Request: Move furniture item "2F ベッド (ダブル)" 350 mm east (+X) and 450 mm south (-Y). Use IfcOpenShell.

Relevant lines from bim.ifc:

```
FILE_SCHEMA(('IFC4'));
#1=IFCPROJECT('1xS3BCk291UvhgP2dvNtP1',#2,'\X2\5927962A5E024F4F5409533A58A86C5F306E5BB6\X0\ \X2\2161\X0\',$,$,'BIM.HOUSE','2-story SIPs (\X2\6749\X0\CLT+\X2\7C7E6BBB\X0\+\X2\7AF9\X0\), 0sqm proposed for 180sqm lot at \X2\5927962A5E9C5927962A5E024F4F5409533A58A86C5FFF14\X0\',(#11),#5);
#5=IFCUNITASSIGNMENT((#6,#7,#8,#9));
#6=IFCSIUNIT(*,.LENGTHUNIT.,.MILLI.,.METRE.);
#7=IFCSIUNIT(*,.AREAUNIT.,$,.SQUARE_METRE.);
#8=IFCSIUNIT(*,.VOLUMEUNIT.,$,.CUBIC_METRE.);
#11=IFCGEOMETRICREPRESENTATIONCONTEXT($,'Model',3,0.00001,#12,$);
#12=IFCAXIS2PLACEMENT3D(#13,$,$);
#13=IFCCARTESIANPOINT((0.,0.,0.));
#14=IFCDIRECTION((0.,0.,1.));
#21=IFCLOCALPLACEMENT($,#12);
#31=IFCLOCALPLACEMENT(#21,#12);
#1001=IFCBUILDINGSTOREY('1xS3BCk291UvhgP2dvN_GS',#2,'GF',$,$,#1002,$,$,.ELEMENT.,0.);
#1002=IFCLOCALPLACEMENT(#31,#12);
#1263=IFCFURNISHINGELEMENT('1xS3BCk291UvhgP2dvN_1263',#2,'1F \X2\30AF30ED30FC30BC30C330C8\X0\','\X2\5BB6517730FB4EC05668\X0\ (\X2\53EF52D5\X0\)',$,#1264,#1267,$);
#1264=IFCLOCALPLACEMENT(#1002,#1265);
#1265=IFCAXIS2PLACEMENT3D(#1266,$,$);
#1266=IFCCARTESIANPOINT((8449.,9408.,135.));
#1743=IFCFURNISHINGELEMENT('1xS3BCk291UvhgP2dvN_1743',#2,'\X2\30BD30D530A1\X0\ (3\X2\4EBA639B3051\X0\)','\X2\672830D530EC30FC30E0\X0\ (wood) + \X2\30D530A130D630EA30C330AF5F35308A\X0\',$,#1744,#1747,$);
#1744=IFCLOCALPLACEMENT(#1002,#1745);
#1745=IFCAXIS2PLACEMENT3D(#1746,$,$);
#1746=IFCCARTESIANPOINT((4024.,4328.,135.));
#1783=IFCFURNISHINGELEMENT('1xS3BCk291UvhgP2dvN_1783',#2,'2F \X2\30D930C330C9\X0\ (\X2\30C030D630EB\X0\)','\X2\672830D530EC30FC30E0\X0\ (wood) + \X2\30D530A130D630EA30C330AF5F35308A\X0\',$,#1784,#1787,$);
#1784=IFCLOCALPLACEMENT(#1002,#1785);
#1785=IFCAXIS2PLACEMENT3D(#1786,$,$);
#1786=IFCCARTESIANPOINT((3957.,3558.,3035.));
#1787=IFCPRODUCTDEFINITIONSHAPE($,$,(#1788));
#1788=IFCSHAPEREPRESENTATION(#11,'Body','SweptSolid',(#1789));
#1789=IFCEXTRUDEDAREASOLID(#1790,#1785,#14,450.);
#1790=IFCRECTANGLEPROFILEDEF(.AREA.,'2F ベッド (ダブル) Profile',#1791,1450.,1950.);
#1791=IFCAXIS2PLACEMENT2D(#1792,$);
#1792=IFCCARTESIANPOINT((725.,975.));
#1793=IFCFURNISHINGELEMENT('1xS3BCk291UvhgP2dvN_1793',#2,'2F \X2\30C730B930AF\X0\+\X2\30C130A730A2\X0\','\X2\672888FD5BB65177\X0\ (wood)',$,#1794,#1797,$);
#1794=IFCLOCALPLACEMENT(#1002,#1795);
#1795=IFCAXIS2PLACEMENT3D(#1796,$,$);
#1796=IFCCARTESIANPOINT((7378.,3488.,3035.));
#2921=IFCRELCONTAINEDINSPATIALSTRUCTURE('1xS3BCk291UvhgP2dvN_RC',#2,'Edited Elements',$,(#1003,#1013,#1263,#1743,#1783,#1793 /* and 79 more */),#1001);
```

```python
import ifcopenshell
import ifcopenshell.api.geometry
import ifcopenshell.util.placement
import ifcopenshell.util.unit

model = ifcopenshell.open("bim.ifc")
unit_scale = ifcopenshell.util.unit.calculate_unit_scale(model)

item = model.by_guid("1xS3BCk291UvhgP2dvN_1783")
matrix = ifcopenshell.util.placement.get_local_placement(item.ObjectPlacement)
matrix[0, 3] += 0.35 / unit_scale
matrix[1, 3] -= 0.45 / unit_scale
ifcopenshell.api.geometry.edit_object_placement(model, product=item, matrix=matrix, is_si=False)

print(ifcopenshell.util.placement.get_local_placement(item.ObjectPlacement).round(3) + 0.0)

model.write("bim_rev.ifc")
```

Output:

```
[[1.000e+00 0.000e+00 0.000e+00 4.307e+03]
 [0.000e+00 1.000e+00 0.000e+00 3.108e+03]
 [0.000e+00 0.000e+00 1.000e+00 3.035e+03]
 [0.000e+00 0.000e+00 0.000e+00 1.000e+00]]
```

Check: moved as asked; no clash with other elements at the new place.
